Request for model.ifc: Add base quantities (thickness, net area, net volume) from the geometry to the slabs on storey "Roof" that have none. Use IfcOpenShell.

First a look at what the model holds.

```python
import ifcopenshell
import ifcopenshell.util.element
import ifcopenshell.util.unit

model = ifcopenshell.open("model.ifc")
print(model.schema)
for unit_type in ("LENGTHUNIT", "AREAUNIT", "VOLUMEUNIT"):
    print(unit_type, ifcopenshell.util.unit.calculate_unit_scale(model, unit_type))
storey = next(s for s in model.by_type("IfcBuildingStorey") if s.Name == "Roof")
slabs = [e for e in ifcopenshell.util.element.get_decomposition(storey) if e.is_a("IfcSlab")]
for e in sorted(slabs, key=lambda e: e.id()):
    print(e.id(), e.is_a(), e.Name, list(ifcopenshell.util.element.get_psets(e, qtos_only=True)), sep=" | ")
```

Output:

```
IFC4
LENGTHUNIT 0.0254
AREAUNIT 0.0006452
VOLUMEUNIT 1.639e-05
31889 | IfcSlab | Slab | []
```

```python
import ifcopenshell
import ifcopenshell.api.pset
import ifcopenshell.geom
import ifcopenshell.util.element
import ifcopenshell.util.shape
import ifcopenshell.util.unit

model = ifcopenshell.open("model.ifc")
unit_scale = ifcopenshell.util.unit.calculate_unit_scale(model)
area_scale = ifcopenshell.util.unit.calculate_unit_scale(model, "AREAUNIT")
volume_scale = ifcopenshell.util.unit.calculate_unit_scale(model, "VOLUMEUNIT")
settings = ifcopenshell.geom.settings()

storey = next(s for s in model.by_type("IfcBuildingStorey") if s.Name == "Roof")
slabs = [e for e in ifcopenshell.util.element.get_decomposition(storey) if e.is_a("IfcSlab")]

for e in sorted(slabs, key=lambda e: e.id()):
    if ifcopenshell.util.element.get_psets(e, qtos_only=True, should_inherit=False):
        continue
    # Geometry comes back in metres, in the element's own axes.
    shape = ifcopenshell.geom.create_shape(settings, e)
    values = {
        "Width": ifcopenshell.util.shape.get_z(shape.geometry) / unit_scale,
        "NetArea": ifcopenshell.util.shape.get_footprint_area(shape.geometry) / area_scale,
        "NetVolume": ifcopenshell.util.shape.get_volume(shape.geometry) / volume_scale,
    }
    qto = ifcopenshell.api.pset.add_qto(model, product=e, name="Qto_SlabBaseQuantities")
    ifcopenshell.api.pset.edit_qto(model, qto=qto, properties=values)
    print(e.id(), {k: round(v, 3) for k, v in values.items()})

model.write("model_rev.ifc")
```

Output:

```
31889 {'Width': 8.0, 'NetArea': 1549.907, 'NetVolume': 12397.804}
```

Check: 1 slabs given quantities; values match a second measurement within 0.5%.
